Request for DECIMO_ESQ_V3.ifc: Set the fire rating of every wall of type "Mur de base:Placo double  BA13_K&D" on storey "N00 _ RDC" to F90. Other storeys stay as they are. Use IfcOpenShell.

First a look at what the model holds.

```python
import ifcopenshell
import ifcopenshell.util.element

model = ifcopenshell.open("DECIMO_ESQ_V3.ifc")
print(model.schema)
storey = next(s for s in model.by_type("IfcBuildingStorey") if s.Name == "N00 _ RDC")
walls = [e for e in ifcopenshell.util.element.get_decomposition(storey) if e.is_a("IfcWall")]
seen = {}
for e in walls:
    element_type = ifcopenshell.util.element.get_type(e)
    key = (element_type.Name if element_type != e and element_type else None, ifcopenshell.util.element.get_pset(e, "Pset_WallCommon", "FireRating"))
    seen[key] = seen.get(key, 0) + 1
for (name, value), count in sorted(seen.items(), key=str):
    print(count, "x", name, "|", value)
```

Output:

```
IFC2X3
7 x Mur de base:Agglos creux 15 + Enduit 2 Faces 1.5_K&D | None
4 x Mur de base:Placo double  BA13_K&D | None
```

```python
import ifcopenshell
import ifcopenshell.api.pset
import ifcopenshell.util.element

model = ifcopenshell.open("DECIMO_ESQ_V3.ifc")

storey = next(s for s in model.by_type("IfcBuildingStorey") if s.Name == "N00 _ RDC")
walls = [e for e in ifcopenshell.util.element.get_decomposition(storey) if e.is_a("IfcWall")]

count = 0
for e in walls:
    element_type = ifcopenshell.util.element.get_type(e)
    if element_type in (None, e) or element_type.Name != "Mur de base:Placo double  BA13_K&D":
        continue
    # add_pset returns the element's existing set when there is one.
    pset = ifcopenshell.api.pset.add_pset(model, product=e, name="Pset_WallCommon")
    ifcopenshell.api.pset.edit_pset(model, pset=pset, properties={"FireRating": "F90"})
    count += 1

print(count, "walls updated")

model.write("DECIMO_ESQ_V3_edited.ifc")
```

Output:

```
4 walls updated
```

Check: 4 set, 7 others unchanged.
